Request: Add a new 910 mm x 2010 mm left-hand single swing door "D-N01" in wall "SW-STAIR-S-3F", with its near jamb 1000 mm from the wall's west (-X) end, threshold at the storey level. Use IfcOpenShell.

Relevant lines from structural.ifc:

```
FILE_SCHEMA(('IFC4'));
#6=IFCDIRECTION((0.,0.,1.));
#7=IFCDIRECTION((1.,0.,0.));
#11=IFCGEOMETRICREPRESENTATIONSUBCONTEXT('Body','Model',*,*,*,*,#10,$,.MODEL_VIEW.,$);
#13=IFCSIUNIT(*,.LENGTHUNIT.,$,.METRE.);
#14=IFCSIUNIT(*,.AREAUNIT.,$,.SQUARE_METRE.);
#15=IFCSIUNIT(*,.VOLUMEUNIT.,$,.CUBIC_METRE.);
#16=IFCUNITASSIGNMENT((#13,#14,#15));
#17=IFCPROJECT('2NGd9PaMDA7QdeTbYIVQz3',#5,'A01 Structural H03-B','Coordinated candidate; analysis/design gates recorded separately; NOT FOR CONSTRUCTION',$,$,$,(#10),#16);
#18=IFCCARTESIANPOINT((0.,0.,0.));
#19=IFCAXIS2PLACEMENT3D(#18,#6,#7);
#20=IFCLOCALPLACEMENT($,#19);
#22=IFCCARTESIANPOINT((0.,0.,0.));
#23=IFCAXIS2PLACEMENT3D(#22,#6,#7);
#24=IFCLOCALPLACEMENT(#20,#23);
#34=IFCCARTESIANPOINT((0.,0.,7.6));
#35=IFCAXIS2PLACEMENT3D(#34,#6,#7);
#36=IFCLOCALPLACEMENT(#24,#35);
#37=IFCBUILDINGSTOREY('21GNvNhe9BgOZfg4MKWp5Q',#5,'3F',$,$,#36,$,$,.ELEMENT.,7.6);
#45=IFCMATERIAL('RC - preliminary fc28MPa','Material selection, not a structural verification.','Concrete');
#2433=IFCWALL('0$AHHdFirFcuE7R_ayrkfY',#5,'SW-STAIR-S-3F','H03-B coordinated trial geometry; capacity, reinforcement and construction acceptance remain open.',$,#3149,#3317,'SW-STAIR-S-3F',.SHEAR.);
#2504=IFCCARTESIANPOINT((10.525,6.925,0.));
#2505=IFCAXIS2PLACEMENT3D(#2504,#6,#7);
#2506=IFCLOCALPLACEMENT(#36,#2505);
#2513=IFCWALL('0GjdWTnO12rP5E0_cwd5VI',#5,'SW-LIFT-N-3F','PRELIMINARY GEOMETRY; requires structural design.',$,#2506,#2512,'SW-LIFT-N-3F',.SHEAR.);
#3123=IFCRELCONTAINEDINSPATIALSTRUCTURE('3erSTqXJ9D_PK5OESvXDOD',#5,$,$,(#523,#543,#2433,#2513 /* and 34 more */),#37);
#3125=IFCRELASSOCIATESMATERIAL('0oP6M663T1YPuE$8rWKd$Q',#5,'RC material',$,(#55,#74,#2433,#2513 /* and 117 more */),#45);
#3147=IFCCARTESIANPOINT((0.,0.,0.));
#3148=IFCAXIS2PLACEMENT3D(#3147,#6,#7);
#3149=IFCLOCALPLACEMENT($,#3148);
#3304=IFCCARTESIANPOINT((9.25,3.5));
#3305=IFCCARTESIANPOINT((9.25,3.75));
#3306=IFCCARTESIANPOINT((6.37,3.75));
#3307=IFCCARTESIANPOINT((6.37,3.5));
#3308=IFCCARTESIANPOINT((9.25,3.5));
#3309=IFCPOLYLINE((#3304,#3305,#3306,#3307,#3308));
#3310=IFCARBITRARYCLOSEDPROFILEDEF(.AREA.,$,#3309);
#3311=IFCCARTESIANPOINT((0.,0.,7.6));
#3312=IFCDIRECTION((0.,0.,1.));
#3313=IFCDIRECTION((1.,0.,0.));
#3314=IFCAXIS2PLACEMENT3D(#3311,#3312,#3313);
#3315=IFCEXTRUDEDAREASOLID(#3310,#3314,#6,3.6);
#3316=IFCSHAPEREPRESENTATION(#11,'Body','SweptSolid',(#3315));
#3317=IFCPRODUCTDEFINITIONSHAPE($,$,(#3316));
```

```python
import numpy as np
import ifcopenshell
import ifcopenshell.api.feature
import ifcopenshell.api.geometry
import ifcopenshell.api.root
import ifcopenshell.api.spatial
import ifcopenshell.geom
import ifcopenshell.util.element
import ifcopenshell.util.placement
import ifcopenshell.util.representation
import ifcopenshell.util.shape
import ifcopenshell.util.unit

model = ifcopenshell.open("structural.ifc")
unit_scale = ifcopenshell.util.unit.calculate_unit_scale(model)
settings = ifcopenshell.geom.settings()


def volume(element):
    """Net volume in cubic metres, openings subtracted."""
    shape = ifcopenshell.geom.create_shape(settings, element)
    return ifcopenshell.util.shape.get_volume(shape.geometry)


wall = model.by_guid("0$AHHdFirFcuE7R_ayrkfY")
storey = ifcopenshell.util.element.get_container(wall, ifc_class="IfcBuildingStorey")
context = ifcopenshell.util.representation.get_context(model, "Model", "Body", "MODEL_VIEW")
before = volume(wall)

width, height, from_end, sill = 0.91, 2.01, 1, 0.0  # metres

# The wall runs along its own X axis, and the end named is its -X end.
wall_shape = ifcopenshell.geom.create_shape(settings, wall)
x, y, z = ifcopenshell.util.shape.get_vertices(wall_shape.geometry).T
start = x.min() + from_end
face, thickness = float(y.min()), float(y.max() - y.min())
wall_matrix = ifcopenshell.util.placement.get_local_placement(wall.ObjectPlacement)
level = ifcopenshell.util.placement.get_local_placement(storey.ObjectPlacement)[2, 3]


def in_wall(x, y):
    """Placement at x, y metres in the wall's axes, at sill height."""
    matrix = wall_matrix.copy()
    matrix[:, 3] = wall_matrix @ np.array([x / unit_scale, y / unit_scale, 0.0, 1.0])
    matrix[2, 3] = level + sill / unit_scale
    return matrix


# Opening: a box that overshoots both wall faces by 50 mm.
opening = ifcopenshell.api.root.create_entity(model, ifc_class="IfcOpeningElement", predefined_type="OPENING")
box = ifcopenshell.api.geometry.add_wall_representation(
    model, context=context, length=width, height=height, thickness=thickness + 0.1
)
ifcopenshell.api.geometry.assign_representation(model, product=opening, representation=box)
ifcopenshell.api.geometry.edit_object_placement(model, product=opening, matrix=in_wall(start, face - 0.05), is_si=False)
ifcopenshell.api.feature.add_feature(model, feature=opening, element=wall)

door = ifcopenshell.api.root.create_entity(model, ifc_class="IfcDoor", name="D-N01", predefined_type="DOOR")
door.OverallWidth, door.OverallHeight = width / unit_scale, height / unit_scale
door.OperationType = "SINGLE_SWING_LEFT"
body = ifcopenshell.api.geometry.add_door_representation(
    model,
    context=context,
    overall_width=door.OverallWidth,
    overall_height=door.OverallHeight,
    operation_type="SINGLE_SWING_LEFT",
    lining_properties={"LiningDepth": thickness / unit_scale, "ThresholdDepth": thickness / unit_scale},
)
ifcopenshell.api.geometry.assign_representation(model, product=door, representation=body)
ifcopenshell.api.spatial.assign_container(model, products=[door], relating_structure=storey)
ifcopenshell.api.feature.add_filling(model, opening=opening, element=door)

# The lining spans the wall, so the door starts at the wall face.
ifcopenshell.api.geometry.edit_object_placement(model, product=door, matrix=in_wall(start, face), is_si=False)

after = volume(wall)

print(f"wall volume {before:.3f} -> {after:.3f} m3")

model.write("structural_updated.ifc")
```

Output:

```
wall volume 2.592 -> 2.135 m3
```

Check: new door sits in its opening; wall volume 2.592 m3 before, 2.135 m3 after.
